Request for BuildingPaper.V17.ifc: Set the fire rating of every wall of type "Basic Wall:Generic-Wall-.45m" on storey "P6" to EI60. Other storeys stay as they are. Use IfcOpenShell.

First a look at what the model holds.

```python
import ifcopenshell
import ifcopenshell.util.element

model = ifcopenshell.open("BuildingPaper.V17.ifc")
print(model.schema)
storey = next(s for s in model.by_type("IfcBuildingStorey") if s.Name == "P6")
walls = [e for e in ifcopenshell.util.element.get_decomposition(storey) if e.is_a("IfcWall")]
seen = {}
for e in walls:
    element_type = ifcopenshell.util.element.get_type(e)
    key = (element_type.Name if element_type != e and element_type else None, ifcopenshell.util.element.get_pset(e, "Pset_WallCommon", "FireRating"))
    seen[key] = seen.get(key, 0) + 1
for (name, value), count in sorted(seen.items(), key=str):
    print(count, "x", name, "|", value)
```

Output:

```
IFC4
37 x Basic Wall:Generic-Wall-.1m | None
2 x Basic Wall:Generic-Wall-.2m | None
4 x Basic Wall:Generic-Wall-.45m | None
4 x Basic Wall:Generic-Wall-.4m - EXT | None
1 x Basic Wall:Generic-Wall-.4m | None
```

```python
import ifcopenshell
import ifcopenshell.api.pset
import ifcopenshell.util.element

model = ifcopenshell.open("BuildingPaper.V17.ifc")

storey = next(s for s in model.by_type("IfcBuildingStorey") if s.Name == "P6")
walls = [e for e in ifcopenshell.util.element.get_decomposition(storey) if e.is_a("IfcWall")]

count = 0
for e in walls:
    element_type = ifcopenshell.util.element.get_type(e)
    if element_type in (None, e) or element_type.Name != "Basic Wall:Generic-Wall-.45m":
        continue
    # add_pset returns the element's existing set when there is one.
    pset = ifcopenshell.api.pset.add_pset(model, product=e, name="Pset_WallCommon")
    ifcopenshell.api.pset.edit_pset(model, pset=pset, properties={"FireRating": "EI60"})
    count += 1

print(count, "walls updated")

model.write("BuildingPaper.V17_v2.ifc")
```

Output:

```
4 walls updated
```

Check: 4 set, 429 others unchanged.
